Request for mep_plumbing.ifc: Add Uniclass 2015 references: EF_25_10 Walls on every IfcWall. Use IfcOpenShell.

First a look at what the model holds.

```python
import ifcopenshell

model = ifcopenshell.open("mep_plumbing.ifc")
print(model.schema)
print("classifications:", [c.Name for c in model.by_type("IfcClassification")])
for ifc_class in ("IfcDoor", "IfcRoof", "IfcStair", "IfcWall", "IfcWindow"):
    print(ifc_class, len(model.by_type(ifc_class)))
```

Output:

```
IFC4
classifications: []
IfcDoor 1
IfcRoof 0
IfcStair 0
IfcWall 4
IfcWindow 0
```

```python
import ifcopenshell
import ifcopenshell.api.classification

model = ifcopenshell.open("mep_plumbing.ifc")

system = ifcopenshell.api.classification.add_classification(model, classification="Uniclass 2015")

codes = {
    "IfcWall": ("EF_25_10", "Walls"),
}
for ifc_class, (code, name) in codes.items():
    products = model.by_type(ifc_class)
    ifcopenshell.api.classification.add_reference(
        model, products=products, classification=system, identification=code, name=name
    )
    print(code, len(products))

model.write("mep_plumbing_edited.ifc")
```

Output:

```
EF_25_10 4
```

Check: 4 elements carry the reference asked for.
